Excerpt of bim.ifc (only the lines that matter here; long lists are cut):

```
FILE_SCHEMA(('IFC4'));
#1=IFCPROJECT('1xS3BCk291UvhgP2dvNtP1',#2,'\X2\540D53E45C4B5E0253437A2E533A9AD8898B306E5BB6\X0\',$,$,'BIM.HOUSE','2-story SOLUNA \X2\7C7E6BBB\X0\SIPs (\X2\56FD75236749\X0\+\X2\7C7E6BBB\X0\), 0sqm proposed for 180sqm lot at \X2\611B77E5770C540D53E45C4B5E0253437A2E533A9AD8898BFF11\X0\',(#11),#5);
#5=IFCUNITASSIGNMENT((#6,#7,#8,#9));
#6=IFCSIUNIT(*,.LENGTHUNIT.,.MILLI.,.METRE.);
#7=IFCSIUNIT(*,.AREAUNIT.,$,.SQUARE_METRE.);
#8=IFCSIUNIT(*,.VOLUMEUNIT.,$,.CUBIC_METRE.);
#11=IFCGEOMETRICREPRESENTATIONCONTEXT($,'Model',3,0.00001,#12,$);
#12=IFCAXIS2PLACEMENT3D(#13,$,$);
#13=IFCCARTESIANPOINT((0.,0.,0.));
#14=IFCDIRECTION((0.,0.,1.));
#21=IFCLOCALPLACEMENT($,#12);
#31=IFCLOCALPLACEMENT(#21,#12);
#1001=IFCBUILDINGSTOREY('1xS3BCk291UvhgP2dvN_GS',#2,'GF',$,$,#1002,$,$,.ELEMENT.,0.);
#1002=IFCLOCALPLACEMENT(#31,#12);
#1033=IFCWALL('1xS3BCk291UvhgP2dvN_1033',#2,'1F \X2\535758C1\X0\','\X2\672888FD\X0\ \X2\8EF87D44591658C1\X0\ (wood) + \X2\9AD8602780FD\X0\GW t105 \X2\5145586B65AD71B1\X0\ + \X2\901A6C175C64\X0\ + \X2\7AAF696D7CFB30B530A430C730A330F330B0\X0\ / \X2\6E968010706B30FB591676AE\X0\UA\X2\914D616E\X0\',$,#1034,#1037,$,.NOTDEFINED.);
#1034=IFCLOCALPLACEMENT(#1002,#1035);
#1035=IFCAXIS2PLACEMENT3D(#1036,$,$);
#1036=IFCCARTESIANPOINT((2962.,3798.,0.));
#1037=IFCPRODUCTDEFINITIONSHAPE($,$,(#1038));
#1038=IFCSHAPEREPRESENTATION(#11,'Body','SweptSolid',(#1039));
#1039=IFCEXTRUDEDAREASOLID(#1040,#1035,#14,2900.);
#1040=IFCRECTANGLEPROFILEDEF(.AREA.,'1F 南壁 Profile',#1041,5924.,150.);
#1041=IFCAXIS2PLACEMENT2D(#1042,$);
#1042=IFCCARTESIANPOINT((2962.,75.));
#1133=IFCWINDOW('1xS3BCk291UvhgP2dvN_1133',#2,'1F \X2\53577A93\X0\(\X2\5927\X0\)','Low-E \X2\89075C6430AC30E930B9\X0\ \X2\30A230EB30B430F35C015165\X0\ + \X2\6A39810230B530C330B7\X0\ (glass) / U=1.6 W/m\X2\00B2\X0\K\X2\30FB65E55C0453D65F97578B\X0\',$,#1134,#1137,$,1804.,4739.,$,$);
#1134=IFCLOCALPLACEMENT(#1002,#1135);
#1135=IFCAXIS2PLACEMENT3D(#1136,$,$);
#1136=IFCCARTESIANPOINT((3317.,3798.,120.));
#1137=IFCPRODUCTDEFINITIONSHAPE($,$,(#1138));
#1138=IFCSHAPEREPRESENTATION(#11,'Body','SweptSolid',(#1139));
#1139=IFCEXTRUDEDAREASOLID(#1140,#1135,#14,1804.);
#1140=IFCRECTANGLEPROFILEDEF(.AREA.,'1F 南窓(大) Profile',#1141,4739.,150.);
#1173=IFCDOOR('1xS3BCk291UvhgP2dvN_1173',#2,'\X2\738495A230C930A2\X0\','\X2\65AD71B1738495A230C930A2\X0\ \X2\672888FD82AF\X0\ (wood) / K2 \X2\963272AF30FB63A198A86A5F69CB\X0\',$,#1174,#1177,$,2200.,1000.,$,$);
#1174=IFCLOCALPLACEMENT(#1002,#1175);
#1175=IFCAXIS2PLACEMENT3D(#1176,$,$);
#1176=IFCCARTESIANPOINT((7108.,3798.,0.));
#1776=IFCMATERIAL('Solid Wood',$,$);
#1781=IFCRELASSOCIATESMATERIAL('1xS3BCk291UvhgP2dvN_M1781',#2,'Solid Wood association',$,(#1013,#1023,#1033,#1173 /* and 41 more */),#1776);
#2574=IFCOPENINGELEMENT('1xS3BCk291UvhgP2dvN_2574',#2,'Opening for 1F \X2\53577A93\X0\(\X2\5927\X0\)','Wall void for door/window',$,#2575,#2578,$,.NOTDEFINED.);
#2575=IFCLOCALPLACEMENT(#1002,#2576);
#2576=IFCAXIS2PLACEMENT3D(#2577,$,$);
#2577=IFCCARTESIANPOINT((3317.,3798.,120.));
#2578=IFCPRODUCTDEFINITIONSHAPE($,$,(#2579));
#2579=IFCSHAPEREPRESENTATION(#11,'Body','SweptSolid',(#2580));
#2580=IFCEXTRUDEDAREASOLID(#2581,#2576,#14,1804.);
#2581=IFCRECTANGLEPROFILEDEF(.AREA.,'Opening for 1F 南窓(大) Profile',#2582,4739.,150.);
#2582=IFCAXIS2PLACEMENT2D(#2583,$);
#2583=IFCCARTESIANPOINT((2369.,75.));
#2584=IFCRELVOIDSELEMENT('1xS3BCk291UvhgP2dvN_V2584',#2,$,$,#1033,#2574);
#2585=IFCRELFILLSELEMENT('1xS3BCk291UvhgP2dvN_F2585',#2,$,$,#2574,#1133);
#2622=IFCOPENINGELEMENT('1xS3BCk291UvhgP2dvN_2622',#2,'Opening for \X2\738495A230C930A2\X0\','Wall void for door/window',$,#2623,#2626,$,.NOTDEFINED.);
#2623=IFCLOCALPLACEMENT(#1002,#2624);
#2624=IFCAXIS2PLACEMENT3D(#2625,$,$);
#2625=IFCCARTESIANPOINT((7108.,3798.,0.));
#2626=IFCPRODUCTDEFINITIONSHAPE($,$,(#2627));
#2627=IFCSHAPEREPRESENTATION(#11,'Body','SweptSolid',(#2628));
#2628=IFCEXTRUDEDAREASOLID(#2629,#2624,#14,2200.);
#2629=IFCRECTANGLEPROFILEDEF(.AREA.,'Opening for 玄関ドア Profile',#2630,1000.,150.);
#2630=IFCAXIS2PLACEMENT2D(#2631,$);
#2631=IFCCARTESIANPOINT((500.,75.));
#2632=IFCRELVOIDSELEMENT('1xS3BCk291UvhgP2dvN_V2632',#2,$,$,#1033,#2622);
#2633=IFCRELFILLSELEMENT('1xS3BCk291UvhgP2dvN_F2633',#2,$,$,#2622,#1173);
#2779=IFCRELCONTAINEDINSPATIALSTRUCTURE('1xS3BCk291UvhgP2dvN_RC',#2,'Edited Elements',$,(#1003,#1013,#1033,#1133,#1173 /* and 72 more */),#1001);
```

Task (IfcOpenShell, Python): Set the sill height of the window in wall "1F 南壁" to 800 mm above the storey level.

```python
import numpy as np
import ifcopenshell
import ifcopenshell.api.geometry
import ifcopenshell.geom
import ifcopenshell.util.element
import ifcopenshell.util.placement
import ifcopenshell.util.shape
import ifcopenshell.util.unit

model = ifcopenshell.open("bim.ifc")
unit_scale = ifcopenshell.util.unit.calculate_unit_scale(model)

window = model.by_guid("1xS3BCk291UvhgP2dvN_1133")
opening = window.FillsVoids[0].RelatingOpeningElement
storey = ifcopenshell.util.element.get_container(window, ifc_class="IfcBuildingStorey")
level = ifcopenshell.util.placement.get_local_placement(storey.ObjectPlacement)[2, 3]

# The opening's origin need not be at the sill, so measure its lowest point.
shape = ifcopenshell.geom.create_shape(ifcopenshell.geom.settings(), opening)
bottom = ifcopenshell.util.shape.get_shape_bottom_elevation(shape, shape.geometry) / unit_scale
dz = level + 0.8 / unit_scale - bottom

shift = np.array([0.0, 0.0, dz])
# The window is not placed relative to its opening, so move both.
for product in (opening, window):
    matrix = ifcopenshell.util.placement.get_local_placement(product.ObjectPlacement)
    matrix[:3, 3] += shift
    ifcopenshell.api.geometry.edit_object_placement(model, product=product, matrix=matrix, is_si=False)

print(f"moved by {dz * unit_scale:+.3f} m")

model.write("bim_updated.ifc")
```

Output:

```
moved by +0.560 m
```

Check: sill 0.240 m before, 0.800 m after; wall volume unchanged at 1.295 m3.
